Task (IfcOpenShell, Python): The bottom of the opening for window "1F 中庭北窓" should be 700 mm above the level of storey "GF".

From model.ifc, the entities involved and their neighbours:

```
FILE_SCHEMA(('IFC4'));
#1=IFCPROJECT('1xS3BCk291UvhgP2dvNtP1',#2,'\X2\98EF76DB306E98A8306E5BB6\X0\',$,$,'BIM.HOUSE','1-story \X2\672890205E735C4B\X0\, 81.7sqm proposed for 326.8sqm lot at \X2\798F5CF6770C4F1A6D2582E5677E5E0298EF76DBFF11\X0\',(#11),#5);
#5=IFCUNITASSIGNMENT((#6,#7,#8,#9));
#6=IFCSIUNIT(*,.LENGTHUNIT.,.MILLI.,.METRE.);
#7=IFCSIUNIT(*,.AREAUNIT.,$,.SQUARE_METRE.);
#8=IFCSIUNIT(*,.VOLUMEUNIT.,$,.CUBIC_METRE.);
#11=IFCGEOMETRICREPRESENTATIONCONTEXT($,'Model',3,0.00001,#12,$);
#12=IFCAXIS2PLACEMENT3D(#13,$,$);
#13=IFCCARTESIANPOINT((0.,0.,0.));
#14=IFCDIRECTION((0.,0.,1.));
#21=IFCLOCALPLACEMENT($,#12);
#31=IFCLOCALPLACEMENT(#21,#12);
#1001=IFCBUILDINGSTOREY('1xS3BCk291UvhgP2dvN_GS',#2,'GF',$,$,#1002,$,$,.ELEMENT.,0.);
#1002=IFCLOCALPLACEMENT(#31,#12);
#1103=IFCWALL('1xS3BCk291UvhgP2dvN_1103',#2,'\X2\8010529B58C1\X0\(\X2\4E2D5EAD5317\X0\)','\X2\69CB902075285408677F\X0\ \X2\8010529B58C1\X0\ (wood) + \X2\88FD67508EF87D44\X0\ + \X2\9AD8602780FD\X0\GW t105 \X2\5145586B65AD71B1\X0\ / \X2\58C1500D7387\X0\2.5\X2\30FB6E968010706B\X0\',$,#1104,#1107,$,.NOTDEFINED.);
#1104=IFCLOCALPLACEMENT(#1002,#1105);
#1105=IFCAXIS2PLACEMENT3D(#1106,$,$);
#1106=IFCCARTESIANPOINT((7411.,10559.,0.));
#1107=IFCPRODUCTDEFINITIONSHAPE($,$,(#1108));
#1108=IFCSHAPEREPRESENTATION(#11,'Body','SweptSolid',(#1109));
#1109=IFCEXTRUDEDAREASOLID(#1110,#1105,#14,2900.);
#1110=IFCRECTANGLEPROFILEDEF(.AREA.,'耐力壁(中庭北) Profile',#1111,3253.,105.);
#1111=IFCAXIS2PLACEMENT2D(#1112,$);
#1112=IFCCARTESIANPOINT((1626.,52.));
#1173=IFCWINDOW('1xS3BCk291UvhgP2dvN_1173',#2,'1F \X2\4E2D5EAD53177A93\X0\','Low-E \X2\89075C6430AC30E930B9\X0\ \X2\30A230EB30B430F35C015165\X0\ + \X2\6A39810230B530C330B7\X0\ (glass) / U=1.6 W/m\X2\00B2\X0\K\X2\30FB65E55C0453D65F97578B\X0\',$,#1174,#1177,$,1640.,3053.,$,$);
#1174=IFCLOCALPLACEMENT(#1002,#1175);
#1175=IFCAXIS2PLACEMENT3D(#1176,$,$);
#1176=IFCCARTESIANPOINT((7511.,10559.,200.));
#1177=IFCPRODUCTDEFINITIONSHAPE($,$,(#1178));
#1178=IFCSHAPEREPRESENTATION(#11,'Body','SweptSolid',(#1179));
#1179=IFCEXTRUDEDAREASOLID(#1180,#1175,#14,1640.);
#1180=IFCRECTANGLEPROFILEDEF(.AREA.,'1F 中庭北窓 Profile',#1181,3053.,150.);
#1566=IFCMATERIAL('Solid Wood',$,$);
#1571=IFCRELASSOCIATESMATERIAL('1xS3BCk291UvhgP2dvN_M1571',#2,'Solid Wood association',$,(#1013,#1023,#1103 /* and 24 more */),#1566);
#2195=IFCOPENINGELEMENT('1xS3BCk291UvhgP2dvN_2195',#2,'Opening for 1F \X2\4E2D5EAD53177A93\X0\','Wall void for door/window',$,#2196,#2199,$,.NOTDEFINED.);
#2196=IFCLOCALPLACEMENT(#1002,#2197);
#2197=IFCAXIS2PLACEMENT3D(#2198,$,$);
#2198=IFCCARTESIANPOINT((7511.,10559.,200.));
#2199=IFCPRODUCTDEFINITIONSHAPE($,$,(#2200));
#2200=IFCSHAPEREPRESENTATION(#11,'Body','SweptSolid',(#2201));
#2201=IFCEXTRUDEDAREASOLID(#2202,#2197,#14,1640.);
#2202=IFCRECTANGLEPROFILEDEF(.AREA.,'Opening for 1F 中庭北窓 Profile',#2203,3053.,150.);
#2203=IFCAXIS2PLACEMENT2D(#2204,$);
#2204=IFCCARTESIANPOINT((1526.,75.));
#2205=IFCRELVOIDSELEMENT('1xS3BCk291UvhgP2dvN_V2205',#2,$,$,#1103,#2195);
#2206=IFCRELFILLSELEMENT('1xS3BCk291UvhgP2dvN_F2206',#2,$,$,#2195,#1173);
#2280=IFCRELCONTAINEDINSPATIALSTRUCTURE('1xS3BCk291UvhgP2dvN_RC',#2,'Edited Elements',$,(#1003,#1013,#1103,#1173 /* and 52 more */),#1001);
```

```python
import numpy as np
import ifcopenshell
import ifcopenshell.api.geometry
import ifcopenshell.geom
import ifcopenshell.util.element
import ifcopenshell.util.placement
import ifcopenshell.util.shape
import ifcopenshell.util.unit

model = ifcopenshell.open("model.ifc")
unit_scale = ifcopenshell.util.unit.calculate_unit_scale(model)

window = model.by_guid("1xS3BCk291UvhgP2dvN_1173")
opening = window.FillsVoids[0].RelatingOpeningElement
storey = ifcopenshell.util.element.get_container(window, ifc_class="IfcBuildingStorey")
level = ifcopenshell.util.placement.get_local_placement(storey.ObjectPlacement)[2, 3]

# The opening's origin need not be at the sill, so measure its lowest point.
shape = ifcopenshell.geom.create_shape(ifcopenshell.geom.settings(), opening)
bottom = ifcopenshell.util.shape.get_shape_bottom_elevation(shape, shape.geometry) / unit_scale
dz = level + 700.0 - bottom

shift = np.array([0.0, 0.0, dz])
# The window is not placed relative to its opening, so move both.
for product in (opening, window):
    matrix = ifcopenshell.util.placement.get_local_placement(product.ObjectPlacement)
    matrix[:3, 3] += shift
    ifcopenshell.api.geometry.edit_object_placement(model, product=product, matrix=matrix, is_si=False)

print(f"moved by {dz * unit_scale:+.3f} m")

model.write("model_edited.ifc")
```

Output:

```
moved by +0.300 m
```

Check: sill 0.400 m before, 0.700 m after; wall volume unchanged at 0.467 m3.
